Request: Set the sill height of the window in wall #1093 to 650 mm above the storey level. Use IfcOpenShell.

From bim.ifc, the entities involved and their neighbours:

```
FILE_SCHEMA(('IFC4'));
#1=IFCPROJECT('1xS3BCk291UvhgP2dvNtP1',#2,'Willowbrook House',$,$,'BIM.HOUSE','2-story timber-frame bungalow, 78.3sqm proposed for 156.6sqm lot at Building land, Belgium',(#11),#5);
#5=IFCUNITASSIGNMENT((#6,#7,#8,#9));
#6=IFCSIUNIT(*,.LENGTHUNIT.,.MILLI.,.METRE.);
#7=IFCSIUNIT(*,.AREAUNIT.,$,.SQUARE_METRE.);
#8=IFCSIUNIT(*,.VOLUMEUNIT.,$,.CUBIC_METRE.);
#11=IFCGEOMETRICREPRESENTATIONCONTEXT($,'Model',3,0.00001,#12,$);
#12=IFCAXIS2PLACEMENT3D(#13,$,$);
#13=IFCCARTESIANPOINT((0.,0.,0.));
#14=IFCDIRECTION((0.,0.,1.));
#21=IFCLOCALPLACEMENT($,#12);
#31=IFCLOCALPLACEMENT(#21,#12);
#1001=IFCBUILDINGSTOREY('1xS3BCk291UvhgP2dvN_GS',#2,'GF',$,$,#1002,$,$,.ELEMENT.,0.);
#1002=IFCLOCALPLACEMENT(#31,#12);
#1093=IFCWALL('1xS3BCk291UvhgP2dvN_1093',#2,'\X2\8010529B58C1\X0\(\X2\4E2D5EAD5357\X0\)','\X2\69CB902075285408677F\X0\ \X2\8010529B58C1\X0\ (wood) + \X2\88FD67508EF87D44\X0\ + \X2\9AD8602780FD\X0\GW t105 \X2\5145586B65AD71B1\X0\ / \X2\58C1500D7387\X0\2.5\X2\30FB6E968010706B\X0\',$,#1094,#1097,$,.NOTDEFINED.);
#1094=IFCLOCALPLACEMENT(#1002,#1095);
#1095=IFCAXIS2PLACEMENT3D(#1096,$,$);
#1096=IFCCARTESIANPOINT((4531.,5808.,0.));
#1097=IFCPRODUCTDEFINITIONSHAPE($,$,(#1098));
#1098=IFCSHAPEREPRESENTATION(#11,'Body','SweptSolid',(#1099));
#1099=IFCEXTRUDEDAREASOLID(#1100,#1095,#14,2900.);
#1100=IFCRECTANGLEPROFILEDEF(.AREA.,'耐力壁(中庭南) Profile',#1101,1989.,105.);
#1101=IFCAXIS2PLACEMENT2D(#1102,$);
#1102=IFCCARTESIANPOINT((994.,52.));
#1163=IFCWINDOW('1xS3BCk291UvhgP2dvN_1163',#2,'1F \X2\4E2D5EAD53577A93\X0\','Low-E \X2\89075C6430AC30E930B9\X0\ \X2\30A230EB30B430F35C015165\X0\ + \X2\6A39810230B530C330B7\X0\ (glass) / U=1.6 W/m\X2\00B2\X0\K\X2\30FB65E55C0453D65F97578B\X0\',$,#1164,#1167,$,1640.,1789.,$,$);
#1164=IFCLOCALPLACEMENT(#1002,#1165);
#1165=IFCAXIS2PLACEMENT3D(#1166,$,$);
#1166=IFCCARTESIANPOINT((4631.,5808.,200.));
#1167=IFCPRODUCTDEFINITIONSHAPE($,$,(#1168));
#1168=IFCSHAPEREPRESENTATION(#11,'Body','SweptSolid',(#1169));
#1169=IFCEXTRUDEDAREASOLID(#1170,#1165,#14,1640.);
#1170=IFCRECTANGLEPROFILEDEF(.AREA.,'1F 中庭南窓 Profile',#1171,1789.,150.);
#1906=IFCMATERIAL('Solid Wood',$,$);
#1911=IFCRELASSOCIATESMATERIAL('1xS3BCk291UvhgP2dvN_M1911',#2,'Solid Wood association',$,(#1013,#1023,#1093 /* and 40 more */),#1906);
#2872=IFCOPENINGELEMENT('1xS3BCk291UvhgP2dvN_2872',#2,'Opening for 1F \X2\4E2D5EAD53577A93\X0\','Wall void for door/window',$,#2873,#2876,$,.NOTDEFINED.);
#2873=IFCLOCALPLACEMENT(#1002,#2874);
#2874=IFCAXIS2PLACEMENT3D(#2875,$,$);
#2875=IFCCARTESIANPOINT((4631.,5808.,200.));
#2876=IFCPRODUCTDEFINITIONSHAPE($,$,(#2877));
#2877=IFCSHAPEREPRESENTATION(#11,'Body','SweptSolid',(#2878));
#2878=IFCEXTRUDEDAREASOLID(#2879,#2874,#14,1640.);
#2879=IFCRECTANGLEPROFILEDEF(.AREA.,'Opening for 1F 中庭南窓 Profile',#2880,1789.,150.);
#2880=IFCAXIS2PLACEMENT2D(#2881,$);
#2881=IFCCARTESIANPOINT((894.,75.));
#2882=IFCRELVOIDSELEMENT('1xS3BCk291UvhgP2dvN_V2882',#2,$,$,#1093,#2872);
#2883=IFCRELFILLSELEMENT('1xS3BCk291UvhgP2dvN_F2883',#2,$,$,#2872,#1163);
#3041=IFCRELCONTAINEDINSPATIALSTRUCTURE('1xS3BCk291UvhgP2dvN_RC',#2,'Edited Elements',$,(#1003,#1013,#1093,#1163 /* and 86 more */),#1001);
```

```python
import numpy as np
import ifcopenshell
import ifcopenshell.api.geometry
import ifcopenshell.geom
import ifcopenshell.util.element
import ifcopenshell.util.placement
import ifcopenshell.util.shape
import ifcopenshell.util.unit

model = ifcopenshell.open("bim.ifc")
unit_scale = ifcopenshell.util.unit.calculate_unit_scale(model)

window = model.by_guid("1xS3BCk291UvhgP2dvN_1163")
opening = window.FillsVoids[0].RelatingOpeningElement
storey = ifcopenshell.util.element.get_container(window, ifc_class="IfcBuildingStorey")
level = ifcopenshell.util.placement.get_local_placement(storey.ObjectPlacement)[2, 3]

# The opening's origin need not be at the sill, so measure its lowest point.
shape = ifcopenshell.geom.create_shape(ifcopenshell.geom.settings(), opening)
bottom = ifcopenshell.util.shape.get_shape_bottom_elevation(shape, shape.geometry) / unit_scale
dz = level + 0.65 / unit_scale - bottom

shift = np.array([0.0, 0.0, dz])
# The window is not placed relative to its opening, so move both.
for product in (opening, window):
    matrix = ifcopenshell.util.placement.get_local_placement(product.ObjectPlacement)
    matrix[:3, 3] += shift
    ifcopenshell.api.geometry.edit_object_placement(model, product=product, matrix=matrix, is_si=False)

print(f"moved by {dz * unit_scale:+.3f} m")

model.write("bim_updated.ifc")
```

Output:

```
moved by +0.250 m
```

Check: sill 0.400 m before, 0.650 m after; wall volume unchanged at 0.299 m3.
